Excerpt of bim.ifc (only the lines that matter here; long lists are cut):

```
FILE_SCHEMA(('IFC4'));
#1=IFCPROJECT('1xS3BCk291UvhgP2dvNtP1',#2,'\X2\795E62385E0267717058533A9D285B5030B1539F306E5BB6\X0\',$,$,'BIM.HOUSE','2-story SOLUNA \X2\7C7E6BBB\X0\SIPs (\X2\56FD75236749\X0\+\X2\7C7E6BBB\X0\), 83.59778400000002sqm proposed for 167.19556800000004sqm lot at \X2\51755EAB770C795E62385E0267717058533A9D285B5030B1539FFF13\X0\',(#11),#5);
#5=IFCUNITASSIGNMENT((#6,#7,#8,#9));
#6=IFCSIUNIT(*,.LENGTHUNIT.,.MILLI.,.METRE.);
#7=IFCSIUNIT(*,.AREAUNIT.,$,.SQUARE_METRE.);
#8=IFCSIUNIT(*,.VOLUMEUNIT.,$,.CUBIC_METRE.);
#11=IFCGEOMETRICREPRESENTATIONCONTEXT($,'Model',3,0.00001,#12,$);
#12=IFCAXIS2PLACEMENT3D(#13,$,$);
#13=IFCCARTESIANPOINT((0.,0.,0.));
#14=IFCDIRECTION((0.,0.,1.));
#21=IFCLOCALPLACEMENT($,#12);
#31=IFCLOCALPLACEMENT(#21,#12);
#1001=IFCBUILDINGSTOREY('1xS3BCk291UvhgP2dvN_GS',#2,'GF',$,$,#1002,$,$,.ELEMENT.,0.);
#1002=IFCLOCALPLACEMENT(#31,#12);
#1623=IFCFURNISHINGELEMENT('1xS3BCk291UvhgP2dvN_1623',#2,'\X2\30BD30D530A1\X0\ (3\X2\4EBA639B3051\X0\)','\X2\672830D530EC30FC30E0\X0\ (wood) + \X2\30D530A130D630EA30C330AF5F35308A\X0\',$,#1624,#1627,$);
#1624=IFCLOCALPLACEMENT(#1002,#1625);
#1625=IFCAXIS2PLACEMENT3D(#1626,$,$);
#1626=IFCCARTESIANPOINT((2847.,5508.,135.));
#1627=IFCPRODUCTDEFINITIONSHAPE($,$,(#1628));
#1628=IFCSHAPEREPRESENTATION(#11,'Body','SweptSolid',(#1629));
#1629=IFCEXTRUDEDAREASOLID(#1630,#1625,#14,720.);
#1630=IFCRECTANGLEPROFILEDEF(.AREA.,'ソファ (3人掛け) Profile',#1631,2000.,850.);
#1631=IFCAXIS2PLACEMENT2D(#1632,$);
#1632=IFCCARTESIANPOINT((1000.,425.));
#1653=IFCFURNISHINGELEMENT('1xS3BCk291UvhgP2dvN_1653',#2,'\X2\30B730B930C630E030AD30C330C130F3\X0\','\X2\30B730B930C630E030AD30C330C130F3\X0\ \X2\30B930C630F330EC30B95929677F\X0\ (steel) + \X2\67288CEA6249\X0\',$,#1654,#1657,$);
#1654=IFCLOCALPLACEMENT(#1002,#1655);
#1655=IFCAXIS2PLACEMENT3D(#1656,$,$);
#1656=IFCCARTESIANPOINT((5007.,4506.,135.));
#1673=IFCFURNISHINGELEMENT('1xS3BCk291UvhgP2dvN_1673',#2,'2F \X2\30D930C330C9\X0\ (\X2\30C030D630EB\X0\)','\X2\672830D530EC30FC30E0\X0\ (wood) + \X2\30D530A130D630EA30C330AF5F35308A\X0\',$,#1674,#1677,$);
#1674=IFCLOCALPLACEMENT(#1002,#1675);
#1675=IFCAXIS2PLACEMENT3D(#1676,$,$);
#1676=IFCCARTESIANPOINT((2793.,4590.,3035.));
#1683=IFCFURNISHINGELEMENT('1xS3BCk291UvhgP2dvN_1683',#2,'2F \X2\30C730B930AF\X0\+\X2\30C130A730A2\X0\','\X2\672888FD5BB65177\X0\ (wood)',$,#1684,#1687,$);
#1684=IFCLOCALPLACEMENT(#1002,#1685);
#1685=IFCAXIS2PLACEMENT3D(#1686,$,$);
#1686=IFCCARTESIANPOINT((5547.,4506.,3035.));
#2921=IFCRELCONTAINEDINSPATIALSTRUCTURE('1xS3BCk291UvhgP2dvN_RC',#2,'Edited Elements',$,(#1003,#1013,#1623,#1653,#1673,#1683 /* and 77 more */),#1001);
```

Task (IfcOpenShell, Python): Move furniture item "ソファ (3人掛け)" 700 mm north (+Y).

```python
import ifcopenshell
import ifcopenshell.api.geometry
import ifcopenshell.util.placement

model = ifcopenshell.open("bim.ifc")

item = model.by_guid("1xS3BCk291UvhgP2dvN_1623")
matrix = ifcopenshell.util.placement.get_local_placement(item.ObjectPlacement)
matrix[1, 3] += 700.0
ifcopenshell.api.geometry.edit_object_placement(model, product=item, matrix=matrix, is_si=False)

print(ifcopenshell.util.placement.get_local_placement(item.ObjectPlacement).round(3) + 0.0)

model.write("bim_updated.ifc")
```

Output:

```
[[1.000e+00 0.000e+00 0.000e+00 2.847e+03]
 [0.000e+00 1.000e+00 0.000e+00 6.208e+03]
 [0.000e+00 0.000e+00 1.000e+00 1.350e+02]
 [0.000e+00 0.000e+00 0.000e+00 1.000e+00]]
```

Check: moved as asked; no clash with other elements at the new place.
